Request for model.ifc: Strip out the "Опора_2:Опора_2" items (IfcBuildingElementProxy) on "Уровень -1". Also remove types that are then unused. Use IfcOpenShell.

First a look at what the model holds.

```python
import ifcopenshell
import ifcopenshell.util.element

model = ifcopenshell.open("model.ifc")
print(model.schema)
storey = next(s for s in model.by_type("IfcBuildingStorey") if s.Name == "Уровень -1")
proxies = [e for e in ifcopenshell.util.element.get_decomposition(storey) if e.is_a("IfcBuildingElementProxy")]
seen = {}
for e in proxies:
    element_type = ifcopenshell.util.element.get_type(e)
    name = element_type.Name if element_type not in (None, e) else None
    seen[name] = seen.get(name, 0) + 1
for name, count in sorted(seen.items(), key=str):
    print(count, "x", name)
```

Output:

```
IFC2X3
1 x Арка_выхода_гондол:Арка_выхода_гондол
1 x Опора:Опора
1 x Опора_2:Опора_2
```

```python
import ifcopenshell
import ifcopenshell.api.root
import ifcopenshell.util.element

model = ifcopenshell.open("model.ifc")

storey = next(s for s in model.by_type("IfcBuildingStorey") if s.Name == "Уровень -1")
proxies = [e for e in ifcopenshell.util.element.get_decomposition(storey) if e.is_a("IfcBuildingElementProxy")]
targets = [e for e in proxies if (t := ifcopenshell.util.element.get_type(e)) not in (None, e) and t.Name == "Опора_2:Опора_2"]
types = {ifcopenshell.util.element.get_type(e) for e in targets} - {None, *targets}

for e in targets:
    ifcopenshell.api.root.remove_product(model, product=e)
print(len(targets), "removed")

unused = [t for t in types if not ifcopenshell.util.element.get_types(t)]
for t in unused:
    ifcopenshell.api.root.remove_product(model, product=t)
print(len(unused), "unused types removed")

model.write("model_v2.ifc")
```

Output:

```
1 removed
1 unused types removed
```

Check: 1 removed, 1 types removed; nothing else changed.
